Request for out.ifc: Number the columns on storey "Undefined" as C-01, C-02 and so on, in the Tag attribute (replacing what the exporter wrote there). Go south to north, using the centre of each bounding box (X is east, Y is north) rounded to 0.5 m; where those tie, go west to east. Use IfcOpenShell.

First a look at what the model holds.

```python
import ifcopenshell
import ifcopenshell.util.element
import ifcopenshell.util.placement

model = ifcopenshell.open("out.ifc")
print(model.schema)
storey = next(s for s in model.by_type("IfcBuildingStorey") if s.Name == "Undefined")
columns = [e for e in ifcopenshell.util.element.get_decomposition(storey) if e.is_a("IfcColumn")]
for e in sorted(columns, key=lambda e: e.id()):
    origin = ifcopenshell.util.placement.get_local_placement(e.ObjectPlacement)[:3, 3]
    print(e.id(), e.Tag, e.Name, origin.round(2) + 0.0, sep=" | ")
```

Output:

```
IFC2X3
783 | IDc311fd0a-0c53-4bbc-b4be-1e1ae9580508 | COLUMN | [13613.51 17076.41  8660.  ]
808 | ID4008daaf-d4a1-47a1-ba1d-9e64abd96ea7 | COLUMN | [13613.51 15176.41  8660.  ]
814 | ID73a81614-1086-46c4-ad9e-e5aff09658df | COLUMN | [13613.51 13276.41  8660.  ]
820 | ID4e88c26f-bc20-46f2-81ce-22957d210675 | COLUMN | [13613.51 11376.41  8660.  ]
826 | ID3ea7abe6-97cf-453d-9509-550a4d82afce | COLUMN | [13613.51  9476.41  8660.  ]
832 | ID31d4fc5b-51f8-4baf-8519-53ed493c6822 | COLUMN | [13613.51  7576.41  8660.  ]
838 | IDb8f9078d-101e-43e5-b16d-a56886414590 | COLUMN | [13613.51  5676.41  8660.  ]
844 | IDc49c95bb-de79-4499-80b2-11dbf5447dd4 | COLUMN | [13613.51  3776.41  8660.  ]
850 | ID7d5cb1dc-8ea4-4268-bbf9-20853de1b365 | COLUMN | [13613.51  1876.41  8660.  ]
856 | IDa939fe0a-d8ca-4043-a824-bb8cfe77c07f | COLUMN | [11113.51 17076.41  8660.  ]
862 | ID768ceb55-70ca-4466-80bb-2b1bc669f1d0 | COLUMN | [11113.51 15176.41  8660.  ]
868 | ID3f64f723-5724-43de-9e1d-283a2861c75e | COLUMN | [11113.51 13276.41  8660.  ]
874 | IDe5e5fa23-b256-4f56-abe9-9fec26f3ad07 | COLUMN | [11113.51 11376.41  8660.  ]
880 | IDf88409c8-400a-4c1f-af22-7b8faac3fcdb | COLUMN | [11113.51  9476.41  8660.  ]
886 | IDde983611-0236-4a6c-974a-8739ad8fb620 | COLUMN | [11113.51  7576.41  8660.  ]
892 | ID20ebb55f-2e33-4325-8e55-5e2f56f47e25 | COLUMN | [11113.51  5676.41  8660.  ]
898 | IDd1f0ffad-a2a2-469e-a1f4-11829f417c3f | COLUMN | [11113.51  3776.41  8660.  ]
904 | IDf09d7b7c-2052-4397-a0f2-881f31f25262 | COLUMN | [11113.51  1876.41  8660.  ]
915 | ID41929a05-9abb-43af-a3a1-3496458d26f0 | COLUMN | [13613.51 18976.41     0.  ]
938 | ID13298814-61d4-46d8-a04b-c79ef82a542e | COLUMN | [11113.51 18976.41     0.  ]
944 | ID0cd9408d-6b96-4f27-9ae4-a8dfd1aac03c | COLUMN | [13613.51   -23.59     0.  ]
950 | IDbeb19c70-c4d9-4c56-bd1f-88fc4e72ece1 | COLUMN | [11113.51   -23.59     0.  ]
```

```python
import ifcopenshell
import ifcopenshell.geom
import ifcopenshell.util.element
import ifcopenshell.util.shape

model = ifcopenshell.open("out.ifc")
settings = ifcopenshell.geom.settings()
settings.set("use-world-coords", True)


def centre(element):
    shape = ifcopenshell.geom.create_shape(settings, element)
    return ifcopenshell.util.shape.get_bbox_centroid(shape.geometry)


storey = next(s for s in model.by_type("IfcBuildingStorey") if s.Name == "Undefined")
columns = [e for e in ifcopenshell.util.element.get_decomposition(storey) if e.is_a("IfcColumn")]

# Insertion points can sit at a corner or the storey origin, so sort by the geometry (in metres).
centres = {e: centre(e) for e in columns}
columns.sort(key=lambda e: (round(centres[e][1] / 0.5), centres[e][0]))

for i, e in enumerate(columns, start=1):
    number = f"C-{i:02d}"
    e.Tag = number
    print(e.id(), number)

model.write("out-out.ifc")
```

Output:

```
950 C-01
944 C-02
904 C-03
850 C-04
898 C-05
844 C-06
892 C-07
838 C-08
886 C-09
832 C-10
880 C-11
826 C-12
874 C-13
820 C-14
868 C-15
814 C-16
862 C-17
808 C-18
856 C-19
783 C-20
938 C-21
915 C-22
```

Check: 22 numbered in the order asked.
